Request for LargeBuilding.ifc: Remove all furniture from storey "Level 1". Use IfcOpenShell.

First a look at what the model holds.

```python
import ifcopenshell
import ifcopenshell.util.element

model = ifcopenshell.open("LargeBuilding.ifc")
print(model.schema)
storey = next(s for s in model.by_type("IfcBuildingStorey") if s.Name == "Level 1")
furniture = [e for e in ifcopenshell.util.element.get_decomposition(storey) if e.is_a("IfcFurnishingElement")]
seen = {}
for e in furniture:
    element_type = ifcopenshell.util.element.get_type(e)
    name = element_type.Name if element_type not in (None, e) else None
    seen[name] = seen.get(name, 0) + 1
for name, count in sorted(seen.items(), key=str):
    print(count, "x", name)
```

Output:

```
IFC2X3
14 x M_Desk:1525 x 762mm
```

```python
import ifcopenshell
import ifcopenshell.api.root
import ifcopenshell.util.element

model = ifcopenshell.open("LargeBuilding.ifc")

storey = next(s for s in model.by_type("IfcBuildingStorey") if s.Name == "Level 1")
furniture = [e for e in ifcopenshell.util.element.get_decomposition(storey) if e.is_a("IfcFurnishingElement")]

for e in furniture:
    ifcopenshell.api.root.remove_product(model, product=e)
print(len(furniture), "removed")

model.write("LargeBuilding_edited.ifc")
```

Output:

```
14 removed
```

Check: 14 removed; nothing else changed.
